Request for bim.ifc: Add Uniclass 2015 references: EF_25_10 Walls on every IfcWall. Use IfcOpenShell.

First a look at what the model holds.

```python
import ifcopenshell

model = ifcopenshell.open("bim.ifc")
print(model.schema)
print("classifications:", [c.Name for c in model.by_type("IfcClassification")])
for ifc_class in ("IfcDoor", "IfcRoof", "IfcStair", "IfcWall", "IfcWindow"):
    print(ifc_class, len(model.by_type(ifc_class)))
```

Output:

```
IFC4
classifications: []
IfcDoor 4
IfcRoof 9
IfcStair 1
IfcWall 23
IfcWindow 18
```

```python
import ifcopenshell
import ifcopenshell.api.classification

model = ifcopenshell.open("bim.ifc")

system = ifcopenshell.api.classification.add_classification(model, classification="Uniclass 2015")

codes = {
    "IfcWall": ("EF_25_10", "Walls"),
}
for ifc_class, (code, name) in codes.items():
    products = model.by_type(ifc_class)
    ifcopenshell.api.classification.add_reference(
        model, products=products, classification=system, identification=code, name=name
    )
    print(code, len(products))

model.write("bim-out.ifc")
```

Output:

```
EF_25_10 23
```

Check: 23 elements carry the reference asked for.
